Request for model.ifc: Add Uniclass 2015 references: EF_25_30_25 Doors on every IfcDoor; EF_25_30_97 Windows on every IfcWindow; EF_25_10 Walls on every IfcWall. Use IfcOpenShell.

First a look at what the model holds.

```python
import ifcopenshell

model = ifcopenshell.open("model.ifc")
print(model.schema)
print("classifications:", [c.Name for c in model.by_type("IfcClassification")])
for ifc_class in ("IfcDoor", "IfcRoof", "IfcStair", "IfcWall", "IfcWindow"):
    print(ifc_class, len(model.by_type(ifc_class)))
```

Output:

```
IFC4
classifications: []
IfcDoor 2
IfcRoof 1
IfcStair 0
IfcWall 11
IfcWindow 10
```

```python
import ifcopenshell
import ifcopenshell.api.classification

model = ifcopenshell.open("model.ifc")

system = ifcopenshell.api.classification.add_classification(model, classification="Uniclass 2015")

codes = {
    "IfcDoor": ("EF_25_30_25", "Doors"),
    "IfcWindow": ("EF_25_30_97", "Windows"),
    "IfcWall": ("EF_25_10", "Walls"),
}
for ifc_class, (code, name) in codes.items():
    products = model.by_type(ifc_class)
    ifcopenshell.api.classification.add_reference(
        model, products=products, classification=system, identification=code, name=name
    )
    print(code, len(products))

model.write("model_edited.ifc")
```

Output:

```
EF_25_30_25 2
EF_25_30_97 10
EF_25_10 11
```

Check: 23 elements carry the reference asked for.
